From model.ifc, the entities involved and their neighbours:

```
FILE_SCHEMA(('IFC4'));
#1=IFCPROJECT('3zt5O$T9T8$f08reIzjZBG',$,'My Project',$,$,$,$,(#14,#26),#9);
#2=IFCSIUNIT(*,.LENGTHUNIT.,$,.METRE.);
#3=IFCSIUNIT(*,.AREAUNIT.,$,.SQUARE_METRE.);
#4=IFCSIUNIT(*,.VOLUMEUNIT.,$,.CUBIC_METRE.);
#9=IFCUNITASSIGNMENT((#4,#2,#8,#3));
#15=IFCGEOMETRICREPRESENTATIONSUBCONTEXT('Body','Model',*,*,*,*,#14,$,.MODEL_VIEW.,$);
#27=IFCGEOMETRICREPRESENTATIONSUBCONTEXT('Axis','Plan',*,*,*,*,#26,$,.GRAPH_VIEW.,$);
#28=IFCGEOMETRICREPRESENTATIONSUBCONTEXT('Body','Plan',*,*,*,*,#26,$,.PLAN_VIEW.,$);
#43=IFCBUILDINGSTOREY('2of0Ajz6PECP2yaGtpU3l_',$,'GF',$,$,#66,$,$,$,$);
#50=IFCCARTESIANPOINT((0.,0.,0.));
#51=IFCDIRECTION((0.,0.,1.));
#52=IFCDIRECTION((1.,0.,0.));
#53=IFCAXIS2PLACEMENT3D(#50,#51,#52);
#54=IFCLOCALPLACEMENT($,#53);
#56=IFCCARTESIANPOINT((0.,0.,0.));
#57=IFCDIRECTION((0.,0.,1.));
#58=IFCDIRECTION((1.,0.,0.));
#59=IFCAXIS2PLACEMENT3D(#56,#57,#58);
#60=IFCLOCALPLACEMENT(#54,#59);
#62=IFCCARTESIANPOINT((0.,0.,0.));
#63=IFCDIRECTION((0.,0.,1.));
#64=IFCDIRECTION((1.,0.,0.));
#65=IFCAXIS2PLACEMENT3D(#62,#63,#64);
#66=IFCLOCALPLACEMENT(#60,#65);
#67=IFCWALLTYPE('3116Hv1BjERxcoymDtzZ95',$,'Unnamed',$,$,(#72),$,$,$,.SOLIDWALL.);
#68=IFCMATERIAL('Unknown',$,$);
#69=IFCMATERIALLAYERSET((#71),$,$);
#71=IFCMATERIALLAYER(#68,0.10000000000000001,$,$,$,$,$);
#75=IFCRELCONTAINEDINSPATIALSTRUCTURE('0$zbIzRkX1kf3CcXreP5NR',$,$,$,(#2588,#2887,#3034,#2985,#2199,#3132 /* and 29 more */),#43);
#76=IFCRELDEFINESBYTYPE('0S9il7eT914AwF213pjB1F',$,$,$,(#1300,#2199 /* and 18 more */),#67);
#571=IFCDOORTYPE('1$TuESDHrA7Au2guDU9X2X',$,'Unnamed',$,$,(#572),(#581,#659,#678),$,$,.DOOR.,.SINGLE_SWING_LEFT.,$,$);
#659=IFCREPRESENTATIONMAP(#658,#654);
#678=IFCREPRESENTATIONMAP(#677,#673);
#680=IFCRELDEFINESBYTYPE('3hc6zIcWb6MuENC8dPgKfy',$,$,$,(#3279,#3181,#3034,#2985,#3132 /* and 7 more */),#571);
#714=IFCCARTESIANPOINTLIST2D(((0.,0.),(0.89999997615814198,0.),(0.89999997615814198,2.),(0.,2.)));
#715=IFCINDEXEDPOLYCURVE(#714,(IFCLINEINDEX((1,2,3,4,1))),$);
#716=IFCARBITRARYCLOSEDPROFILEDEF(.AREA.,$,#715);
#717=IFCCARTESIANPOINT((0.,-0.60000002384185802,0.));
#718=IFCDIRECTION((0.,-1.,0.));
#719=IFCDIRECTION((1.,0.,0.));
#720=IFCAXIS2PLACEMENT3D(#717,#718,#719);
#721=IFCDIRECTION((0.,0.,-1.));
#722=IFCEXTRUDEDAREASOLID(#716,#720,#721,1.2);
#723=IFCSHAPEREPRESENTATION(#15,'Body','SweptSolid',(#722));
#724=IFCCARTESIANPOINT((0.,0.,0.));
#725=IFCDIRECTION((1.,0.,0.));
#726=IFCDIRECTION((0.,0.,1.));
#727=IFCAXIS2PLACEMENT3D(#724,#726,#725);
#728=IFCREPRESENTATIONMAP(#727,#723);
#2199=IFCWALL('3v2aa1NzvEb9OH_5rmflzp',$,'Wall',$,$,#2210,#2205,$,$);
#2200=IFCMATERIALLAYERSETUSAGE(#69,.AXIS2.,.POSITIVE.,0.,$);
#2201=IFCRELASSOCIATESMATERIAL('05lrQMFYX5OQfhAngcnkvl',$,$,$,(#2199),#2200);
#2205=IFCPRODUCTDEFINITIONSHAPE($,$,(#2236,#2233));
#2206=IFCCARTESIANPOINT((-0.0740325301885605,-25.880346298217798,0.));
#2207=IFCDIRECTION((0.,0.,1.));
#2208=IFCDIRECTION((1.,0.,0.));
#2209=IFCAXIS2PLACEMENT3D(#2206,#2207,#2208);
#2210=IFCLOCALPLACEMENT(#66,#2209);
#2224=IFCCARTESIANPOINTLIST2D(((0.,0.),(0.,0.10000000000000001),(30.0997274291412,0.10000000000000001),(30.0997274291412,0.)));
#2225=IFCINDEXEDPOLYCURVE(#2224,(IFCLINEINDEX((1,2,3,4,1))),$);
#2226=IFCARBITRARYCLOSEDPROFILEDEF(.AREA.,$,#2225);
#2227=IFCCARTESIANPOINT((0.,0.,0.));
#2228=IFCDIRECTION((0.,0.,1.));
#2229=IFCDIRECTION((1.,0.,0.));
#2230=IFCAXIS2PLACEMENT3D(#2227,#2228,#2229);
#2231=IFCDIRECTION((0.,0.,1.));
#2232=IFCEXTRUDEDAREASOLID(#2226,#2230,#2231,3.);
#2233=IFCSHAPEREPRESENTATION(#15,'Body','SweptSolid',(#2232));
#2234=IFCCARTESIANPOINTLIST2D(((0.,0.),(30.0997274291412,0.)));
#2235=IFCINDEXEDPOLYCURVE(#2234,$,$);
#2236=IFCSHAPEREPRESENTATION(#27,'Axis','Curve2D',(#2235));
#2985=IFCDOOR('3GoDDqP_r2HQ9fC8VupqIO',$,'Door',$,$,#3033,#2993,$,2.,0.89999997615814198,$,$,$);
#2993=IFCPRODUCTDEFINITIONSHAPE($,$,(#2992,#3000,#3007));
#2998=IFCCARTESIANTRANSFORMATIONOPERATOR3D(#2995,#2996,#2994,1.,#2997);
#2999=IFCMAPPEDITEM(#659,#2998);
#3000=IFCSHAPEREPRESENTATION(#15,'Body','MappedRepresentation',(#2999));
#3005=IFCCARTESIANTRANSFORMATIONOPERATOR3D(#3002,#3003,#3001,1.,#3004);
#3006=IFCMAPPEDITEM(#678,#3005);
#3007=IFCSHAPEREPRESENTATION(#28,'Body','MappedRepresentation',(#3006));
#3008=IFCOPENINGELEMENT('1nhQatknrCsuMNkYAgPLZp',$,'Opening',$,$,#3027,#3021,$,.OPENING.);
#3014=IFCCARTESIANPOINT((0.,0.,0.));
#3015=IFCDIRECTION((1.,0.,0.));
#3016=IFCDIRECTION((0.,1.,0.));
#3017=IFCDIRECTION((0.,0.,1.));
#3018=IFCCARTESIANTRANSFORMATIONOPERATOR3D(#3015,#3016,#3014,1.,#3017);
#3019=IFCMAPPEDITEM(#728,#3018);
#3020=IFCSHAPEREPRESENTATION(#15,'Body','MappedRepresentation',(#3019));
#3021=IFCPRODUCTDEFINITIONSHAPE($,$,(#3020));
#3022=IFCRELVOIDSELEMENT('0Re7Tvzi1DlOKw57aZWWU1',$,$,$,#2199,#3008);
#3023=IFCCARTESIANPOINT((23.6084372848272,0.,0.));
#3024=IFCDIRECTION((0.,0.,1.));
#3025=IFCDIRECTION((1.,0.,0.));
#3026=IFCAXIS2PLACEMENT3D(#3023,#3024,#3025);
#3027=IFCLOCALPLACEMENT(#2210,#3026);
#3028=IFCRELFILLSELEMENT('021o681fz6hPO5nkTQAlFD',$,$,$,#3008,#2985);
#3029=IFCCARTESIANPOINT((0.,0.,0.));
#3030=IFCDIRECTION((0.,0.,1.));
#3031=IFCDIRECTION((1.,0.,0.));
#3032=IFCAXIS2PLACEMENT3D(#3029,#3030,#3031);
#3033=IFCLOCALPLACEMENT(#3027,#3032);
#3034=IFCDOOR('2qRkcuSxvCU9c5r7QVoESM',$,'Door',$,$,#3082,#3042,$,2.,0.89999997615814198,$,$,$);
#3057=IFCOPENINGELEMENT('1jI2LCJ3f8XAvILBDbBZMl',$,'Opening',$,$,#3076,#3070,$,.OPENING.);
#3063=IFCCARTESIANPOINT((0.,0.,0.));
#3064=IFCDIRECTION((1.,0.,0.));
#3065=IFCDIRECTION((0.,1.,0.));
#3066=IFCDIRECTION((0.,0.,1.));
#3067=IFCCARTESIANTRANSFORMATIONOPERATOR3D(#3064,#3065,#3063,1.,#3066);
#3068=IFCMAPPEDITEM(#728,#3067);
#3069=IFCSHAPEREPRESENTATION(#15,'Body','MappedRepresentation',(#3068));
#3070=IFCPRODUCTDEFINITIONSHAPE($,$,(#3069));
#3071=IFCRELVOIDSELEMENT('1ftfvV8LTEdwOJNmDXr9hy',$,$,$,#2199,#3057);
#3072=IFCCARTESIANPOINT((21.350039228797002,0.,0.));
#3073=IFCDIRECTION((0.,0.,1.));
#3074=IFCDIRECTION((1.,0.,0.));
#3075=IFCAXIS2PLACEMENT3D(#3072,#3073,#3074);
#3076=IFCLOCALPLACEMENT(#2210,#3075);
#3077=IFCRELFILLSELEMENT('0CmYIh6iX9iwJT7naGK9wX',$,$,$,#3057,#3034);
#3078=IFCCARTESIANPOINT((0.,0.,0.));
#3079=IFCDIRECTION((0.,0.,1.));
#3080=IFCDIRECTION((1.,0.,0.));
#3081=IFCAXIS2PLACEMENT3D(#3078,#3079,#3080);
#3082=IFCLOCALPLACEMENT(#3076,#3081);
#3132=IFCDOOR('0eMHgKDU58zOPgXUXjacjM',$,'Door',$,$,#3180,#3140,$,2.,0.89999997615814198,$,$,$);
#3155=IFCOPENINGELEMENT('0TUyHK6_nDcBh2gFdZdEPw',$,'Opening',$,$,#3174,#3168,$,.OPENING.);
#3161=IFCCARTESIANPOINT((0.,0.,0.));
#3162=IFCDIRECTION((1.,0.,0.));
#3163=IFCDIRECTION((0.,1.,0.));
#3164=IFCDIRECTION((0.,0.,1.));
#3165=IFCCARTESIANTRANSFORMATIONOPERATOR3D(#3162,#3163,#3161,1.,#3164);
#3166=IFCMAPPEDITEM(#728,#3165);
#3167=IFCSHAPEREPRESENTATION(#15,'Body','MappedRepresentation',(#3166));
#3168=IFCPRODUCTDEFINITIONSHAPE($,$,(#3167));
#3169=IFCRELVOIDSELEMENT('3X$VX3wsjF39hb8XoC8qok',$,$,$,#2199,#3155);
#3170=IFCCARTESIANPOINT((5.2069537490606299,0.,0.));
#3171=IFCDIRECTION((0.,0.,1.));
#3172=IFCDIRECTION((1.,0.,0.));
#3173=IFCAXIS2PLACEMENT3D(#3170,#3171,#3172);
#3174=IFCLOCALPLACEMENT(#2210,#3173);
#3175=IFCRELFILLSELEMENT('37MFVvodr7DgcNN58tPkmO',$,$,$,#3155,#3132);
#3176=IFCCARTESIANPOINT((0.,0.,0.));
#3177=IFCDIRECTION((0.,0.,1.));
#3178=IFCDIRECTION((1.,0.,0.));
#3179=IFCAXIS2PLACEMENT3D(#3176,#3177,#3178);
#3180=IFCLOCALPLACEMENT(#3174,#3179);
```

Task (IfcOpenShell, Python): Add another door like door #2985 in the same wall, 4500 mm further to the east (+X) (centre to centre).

```python
import ifcopenshell
import ifcopenshell.api.feature
import ifcopenshell.api.geometry
import ifcopenshell.api.root
import ifcopenshell.geom
import ifcopenshell.util.element
import ifcopenshell.util.placement
import ifcopenshell.util.shape
import ifcopenshell.util.unit

model = ifcopenshell.open("model.ifc")
unit_scale = ifcopenshell.util.unit.calculate_unit_scale(model)
settings = ifcopenshell.geom.settings()


def volume(element):
    """Net volume in cubic metres, openings subtracted."""
    shape = ifcopenshell.geom.create_shape(settings, element)
    return ifcopenshell.util.shape.get_volume(shape.geometry)


door = model.by_guid("3GoDDqP_r2HQ9fC8VupqIO")
opening = door.FillsVoids[0].RelatingOpeningElement
wall = opening.VoidsElements[0].RelatingBuildingElement
before = volume(wall)
shift = ifcopenshell.util.placement.get_local_placement(wall.ObjectPlacement)[:3, 0] * 4.5 / unit_scale

# copy_class copies the void relationship, type, container and properties, but no geometry.
new_opening = ifcopenshell.api.root.copy_class(model, product=opening)
new_opening.Representation = ifcopenshell.util.element.copy_deep(
    model, opening.Representation, exclude=["IfcGeometricRepresentationContext", "IfcRepresentationMap"]
)
new_door = ifcopenshell.api.root.copy_class(model, product=door)
new_door.Representation = ifcopenshell.util.element.copy_deep(
    model, door.Representation, exclude=["IfcGeometricRepresentationContext", "IfcRepresentationMap"]
)
ifcopenshell.api.feature.add_filling(model, opening=new_opening, element=new_door)

for old, new in ((opening, new_opening), (door, new_door)):
    matrix = ifcopenshell.util.placement.get_local_placement(old.ObjectPlacement)
    matrix[:3, 3] += shift
    ifcopenshell.api.geometry.edit_object_placement(model, product=new, matrix=matrix, is_si=False)

after = volume(wall)

print(f"wall volume {before:.3f} -> {after:.3f} m3")

model.write("model-out.ifc")
```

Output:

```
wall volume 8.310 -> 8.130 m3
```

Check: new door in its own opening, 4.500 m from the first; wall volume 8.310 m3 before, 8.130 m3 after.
